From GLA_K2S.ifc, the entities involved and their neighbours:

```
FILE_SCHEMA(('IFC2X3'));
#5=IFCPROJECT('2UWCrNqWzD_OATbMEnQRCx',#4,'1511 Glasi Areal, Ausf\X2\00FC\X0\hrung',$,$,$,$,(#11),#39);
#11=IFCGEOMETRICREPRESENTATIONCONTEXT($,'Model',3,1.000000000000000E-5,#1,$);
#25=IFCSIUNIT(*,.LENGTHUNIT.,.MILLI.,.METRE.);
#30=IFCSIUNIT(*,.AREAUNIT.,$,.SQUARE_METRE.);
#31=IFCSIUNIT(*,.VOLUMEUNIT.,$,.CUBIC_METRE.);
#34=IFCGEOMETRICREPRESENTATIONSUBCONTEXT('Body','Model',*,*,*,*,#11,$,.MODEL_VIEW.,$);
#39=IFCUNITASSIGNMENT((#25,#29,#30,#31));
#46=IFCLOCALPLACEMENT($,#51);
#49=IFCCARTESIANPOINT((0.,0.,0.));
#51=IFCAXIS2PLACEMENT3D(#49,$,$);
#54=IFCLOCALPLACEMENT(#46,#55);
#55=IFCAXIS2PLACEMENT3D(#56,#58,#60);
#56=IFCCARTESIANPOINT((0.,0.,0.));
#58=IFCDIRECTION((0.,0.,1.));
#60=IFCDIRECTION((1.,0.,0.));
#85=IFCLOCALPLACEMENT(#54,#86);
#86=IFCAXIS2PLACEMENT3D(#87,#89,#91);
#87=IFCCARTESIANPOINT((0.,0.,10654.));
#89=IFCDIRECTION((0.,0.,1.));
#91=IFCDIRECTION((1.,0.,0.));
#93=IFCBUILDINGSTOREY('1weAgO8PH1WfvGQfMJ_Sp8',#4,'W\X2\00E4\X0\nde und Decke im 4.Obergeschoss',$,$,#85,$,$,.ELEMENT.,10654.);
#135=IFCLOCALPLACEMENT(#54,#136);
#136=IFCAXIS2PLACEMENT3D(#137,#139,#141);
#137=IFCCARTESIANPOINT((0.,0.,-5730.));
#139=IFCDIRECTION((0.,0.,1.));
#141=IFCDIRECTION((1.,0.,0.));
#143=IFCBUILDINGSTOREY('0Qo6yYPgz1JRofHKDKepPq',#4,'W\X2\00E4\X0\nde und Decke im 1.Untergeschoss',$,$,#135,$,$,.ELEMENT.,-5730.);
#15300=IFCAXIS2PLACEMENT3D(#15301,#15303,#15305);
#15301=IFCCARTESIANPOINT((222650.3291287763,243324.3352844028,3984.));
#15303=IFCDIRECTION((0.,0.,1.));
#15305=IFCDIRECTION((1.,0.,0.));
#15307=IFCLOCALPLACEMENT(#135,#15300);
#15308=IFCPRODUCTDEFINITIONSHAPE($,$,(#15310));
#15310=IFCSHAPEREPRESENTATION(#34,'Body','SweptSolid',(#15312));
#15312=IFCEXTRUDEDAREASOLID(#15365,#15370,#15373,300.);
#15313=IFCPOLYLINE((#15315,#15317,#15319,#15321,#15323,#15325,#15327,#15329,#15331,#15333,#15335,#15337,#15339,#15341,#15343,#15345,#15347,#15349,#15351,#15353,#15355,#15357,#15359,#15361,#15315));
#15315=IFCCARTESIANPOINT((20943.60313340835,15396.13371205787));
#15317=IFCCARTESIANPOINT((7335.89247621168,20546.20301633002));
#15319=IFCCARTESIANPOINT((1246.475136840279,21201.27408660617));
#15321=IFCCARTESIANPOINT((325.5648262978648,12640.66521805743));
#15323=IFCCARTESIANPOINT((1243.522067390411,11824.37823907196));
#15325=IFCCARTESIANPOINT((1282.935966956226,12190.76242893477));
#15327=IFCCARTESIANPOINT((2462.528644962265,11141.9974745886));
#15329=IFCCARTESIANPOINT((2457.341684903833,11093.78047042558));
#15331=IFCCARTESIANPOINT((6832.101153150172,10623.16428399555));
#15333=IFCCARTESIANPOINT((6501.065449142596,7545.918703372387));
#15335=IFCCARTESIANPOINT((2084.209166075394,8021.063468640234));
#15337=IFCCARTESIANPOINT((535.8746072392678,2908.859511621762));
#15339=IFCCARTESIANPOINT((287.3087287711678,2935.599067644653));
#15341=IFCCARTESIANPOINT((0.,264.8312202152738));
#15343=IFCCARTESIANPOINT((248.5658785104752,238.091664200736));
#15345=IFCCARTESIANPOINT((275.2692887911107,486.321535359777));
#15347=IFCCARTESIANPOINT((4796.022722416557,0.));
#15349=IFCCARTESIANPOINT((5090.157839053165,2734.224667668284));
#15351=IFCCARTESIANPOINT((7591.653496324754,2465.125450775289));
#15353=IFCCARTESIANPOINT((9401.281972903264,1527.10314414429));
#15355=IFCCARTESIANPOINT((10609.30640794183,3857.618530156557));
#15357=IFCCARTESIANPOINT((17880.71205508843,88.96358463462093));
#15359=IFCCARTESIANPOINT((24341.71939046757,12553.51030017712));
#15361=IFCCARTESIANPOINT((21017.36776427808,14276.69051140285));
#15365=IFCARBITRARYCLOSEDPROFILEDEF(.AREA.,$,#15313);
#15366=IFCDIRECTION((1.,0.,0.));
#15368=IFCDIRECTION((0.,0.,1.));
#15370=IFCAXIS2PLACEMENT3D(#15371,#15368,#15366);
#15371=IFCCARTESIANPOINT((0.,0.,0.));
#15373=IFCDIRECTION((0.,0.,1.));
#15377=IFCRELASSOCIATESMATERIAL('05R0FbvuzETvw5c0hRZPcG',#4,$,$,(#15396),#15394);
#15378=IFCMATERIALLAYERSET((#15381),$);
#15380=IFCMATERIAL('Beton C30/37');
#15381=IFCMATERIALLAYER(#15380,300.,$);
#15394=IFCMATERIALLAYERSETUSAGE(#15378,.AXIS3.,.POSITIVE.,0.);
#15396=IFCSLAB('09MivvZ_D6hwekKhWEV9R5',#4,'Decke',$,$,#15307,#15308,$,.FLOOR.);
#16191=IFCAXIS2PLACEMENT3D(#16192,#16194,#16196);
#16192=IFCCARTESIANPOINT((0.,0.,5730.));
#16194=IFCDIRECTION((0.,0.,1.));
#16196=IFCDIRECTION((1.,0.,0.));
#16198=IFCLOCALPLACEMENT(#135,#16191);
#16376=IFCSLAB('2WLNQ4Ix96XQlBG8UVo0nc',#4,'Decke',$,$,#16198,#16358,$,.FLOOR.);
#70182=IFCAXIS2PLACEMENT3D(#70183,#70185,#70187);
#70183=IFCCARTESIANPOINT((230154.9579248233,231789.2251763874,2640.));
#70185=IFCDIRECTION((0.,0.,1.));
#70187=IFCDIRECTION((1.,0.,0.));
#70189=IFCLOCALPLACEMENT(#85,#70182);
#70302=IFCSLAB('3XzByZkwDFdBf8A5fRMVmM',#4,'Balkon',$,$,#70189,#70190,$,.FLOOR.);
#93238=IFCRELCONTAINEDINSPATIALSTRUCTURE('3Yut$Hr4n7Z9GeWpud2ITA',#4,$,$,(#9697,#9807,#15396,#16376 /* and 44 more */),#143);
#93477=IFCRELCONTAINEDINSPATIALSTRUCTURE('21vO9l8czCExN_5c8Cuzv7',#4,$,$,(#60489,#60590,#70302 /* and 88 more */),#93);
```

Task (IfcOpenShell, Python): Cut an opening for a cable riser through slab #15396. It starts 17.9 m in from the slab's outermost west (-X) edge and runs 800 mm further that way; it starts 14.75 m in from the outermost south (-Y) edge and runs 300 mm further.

```python
import numpy as np
import ifcopenshell
import ifcopenshell.api.feature
import ifcopenshell.api.geometry
import ifcopenshell.api.root
import ifcopenshell.geom
import ifcopenshell.util.placement
import ifcopenshell.util.representation
import ifcopenshell.util.shape
import ifcopenshell.util.unit

model = ifcopenshell.open("GLA_K2S.ifc")
unit_scale = ifcopenshell.util.unit.calculate_unit_scale(model)
settings = ifcopenshell.geom.settings()


def volume(element):
    """Net volume in cubic metres, openings subtracted."""
    shape = ifcopenshell.geom.create_shape(settings, element)
    return ifcopenshell.util.shape.get_volume(shape.geometry)


slab = model.by_guid("09MivvZ_D6hwekKhWEV9R5")
before = volume(slab)

# Extent in the slab's own axes, in metres. The edges named are its -X and -Y sides.
slab_shape = ifcopenshell.geom.create_shape(settings, slab)
vertices = ifcopenshell.util.shape.get_vertices(slab_shape.geometry)
x_min, y_min, bottom = vertices.min(axis=0)
top = vertices[:, 2].max()

opening = ifcopenshell.api.root.create_entity(model, ifc_class="IfcOpeningElement", name="Cable riser opening")
context = ifcopenshell.util.representation.get_context(model, "Model", "Body", "MODEL_VIEW")
width, depth = 0.8, 0.3
outline = [(0.0, 0.0), (width, 0.0), (width, depth), (0.0, depth), (0.0, 0.0)]
# Overshoot both faces by 50 mm so the cut is clean.
shape = ifcopenshell.api.geometry.add_slab_representation(
    model, context=context, depth=top - bottom + 0.1, polyline=outline
)
ifcopenshell.api.geometry.assign_representation(model, product=opening, representation=shape)

matrix = ifcopenshell.util.placement.get_local_placement(slab.ObjectPlacement)
matrix[:, 3] = matrix @ np.append(np.array([x_min + 17.9, y_min + 14.75, bottom - 0.05]) / unit_scale, 1.0)
ifcopenshell.api.geometry.edit_object_placement(model, product=opening, matrix=matrix, is_si=False)
ifcopenshell.api.feature.add_feature(model, feature=opening, element=slab)

after = volume(slab)

print(f"slab volume {before:.3f} -> {after:.3f} m3")

model.write("GLA_K2S_edited.ifc")
```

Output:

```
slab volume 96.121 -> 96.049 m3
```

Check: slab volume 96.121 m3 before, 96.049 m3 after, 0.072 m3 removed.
